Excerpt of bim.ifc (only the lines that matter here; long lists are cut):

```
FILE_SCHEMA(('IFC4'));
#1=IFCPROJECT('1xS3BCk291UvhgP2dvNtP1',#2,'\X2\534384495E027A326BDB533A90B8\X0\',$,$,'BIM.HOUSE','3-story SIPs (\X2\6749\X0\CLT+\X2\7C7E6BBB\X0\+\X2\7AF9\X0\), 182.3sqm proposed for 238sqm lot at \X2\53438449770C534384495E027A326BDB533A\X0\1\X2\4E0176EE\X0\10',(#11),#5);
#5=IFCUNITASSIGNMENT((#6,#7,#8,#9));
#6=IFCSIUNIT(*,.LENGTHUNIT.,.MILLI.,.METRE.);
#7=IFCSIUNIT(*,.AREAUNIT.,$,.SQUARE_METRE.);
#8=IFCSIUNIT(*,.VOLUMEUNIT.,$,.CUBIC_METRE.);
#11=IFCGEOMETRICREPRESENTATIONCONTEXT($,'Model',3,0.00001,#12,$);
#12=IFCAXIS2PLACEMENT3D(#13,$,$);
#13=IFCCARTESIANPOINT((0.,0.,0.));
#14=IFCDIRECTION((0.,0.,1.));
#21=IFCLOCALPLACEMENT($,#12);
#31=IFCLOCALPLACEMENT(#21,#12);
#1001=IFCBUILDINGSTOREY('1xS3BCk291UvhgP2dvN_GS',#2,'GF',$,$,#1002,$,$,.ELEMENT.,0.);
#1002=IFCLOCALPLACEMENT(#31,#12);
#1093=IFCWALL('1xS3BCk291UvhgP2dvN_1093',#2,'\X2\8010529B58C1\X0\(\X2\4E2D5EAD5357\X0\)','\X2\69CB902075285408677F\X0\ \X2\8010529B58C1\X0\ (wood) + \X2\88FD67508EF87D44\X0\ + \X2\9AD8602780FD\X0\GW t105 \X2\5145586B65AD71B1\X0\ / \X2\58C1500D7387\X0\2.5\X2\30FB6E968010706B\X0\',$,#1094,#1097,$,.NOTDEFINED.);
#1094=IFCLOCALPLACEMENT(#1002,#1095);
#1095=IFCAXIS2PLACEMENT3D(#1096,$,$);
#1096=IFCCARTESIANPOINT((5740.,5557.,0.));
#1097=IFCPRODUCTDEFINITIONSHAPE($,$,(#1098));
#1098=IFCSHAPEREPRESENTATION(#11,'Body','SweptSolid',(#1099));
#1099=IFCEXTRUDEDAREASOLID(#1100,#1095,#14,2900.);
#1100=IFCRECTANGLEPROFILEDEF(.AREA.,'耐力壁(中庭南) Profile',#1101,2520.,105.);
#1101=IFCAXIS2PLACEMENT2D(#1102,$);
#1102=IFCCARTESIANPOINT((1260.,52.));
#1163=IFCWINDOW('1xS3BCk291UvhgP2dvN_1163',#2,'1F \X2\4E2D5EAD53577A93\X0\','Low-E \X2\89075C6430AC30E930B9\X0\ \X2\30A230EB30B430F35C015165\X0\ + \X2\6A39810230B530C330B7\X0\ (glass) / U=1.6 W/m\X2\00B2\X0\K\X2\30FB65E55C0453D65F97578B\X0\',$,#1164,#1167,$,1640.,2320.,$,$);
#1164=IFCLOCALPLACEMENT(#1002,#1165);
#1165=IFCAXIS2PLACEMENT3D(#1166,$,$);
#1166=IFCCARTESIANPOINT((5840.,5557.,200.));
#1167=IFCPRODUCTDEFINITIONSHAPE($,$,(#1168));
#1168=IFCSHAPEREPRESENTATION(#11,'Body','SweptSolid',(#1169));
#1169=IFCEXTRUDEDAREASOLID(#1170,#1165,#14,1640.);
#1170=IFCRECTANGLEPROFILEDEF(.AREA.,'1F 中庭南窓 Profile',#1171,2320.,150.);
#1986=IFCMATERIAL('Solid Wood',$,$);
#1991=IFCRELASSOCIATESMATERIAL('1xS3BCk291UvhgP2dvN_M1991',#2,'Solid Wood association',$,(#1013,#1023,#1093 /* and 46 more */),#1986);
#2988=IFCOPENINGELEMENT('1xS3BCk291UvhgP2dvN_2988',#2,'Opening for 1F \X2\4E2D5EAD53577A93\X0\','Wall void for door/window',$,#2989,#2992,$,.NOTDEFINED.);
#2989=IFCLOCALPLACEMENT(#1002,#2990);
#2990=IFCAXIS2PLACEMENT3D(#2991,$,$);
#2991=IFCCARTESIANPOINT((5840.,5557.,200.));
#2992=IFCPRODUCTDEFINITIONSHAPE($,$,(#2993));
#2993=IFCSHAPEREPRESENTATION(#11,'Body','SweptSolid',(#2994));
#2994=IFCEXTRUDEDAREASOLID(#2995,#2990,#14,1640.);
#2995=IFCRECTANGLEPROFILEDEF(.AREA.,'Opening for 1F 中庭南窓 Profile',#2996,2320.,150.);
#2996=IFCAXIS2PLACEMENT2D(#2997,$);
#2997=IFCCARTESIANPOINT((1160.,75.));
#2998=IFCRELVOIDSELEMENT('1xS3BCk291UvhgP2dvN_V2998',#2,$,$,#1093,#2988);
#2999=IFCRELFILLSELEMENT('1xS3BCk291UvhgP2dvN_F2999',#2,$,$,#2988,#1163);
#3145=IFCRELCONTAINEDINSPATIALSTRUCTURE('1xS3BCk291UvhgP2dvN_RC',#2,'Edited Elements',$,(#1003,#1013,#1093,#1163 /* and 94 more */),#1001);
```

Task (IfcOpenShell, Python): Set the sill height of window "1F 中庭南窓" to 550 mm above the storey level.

```python
import numpy as np
import ifcopenshell
import ifcopenshell.api.geometry
import ifcopenshell.geom
import ifcopenshell.util.element
import ifcopenshell.util.placement
import ifcopenshell.util.shape
import ifcopenshell.util.unit

model = ifcopenshell.open("bim.ifc")
unit_scale = ifcopenshell.util.unit.calculate_unit_scale(model)

window = model.by_guid("1xS3BCk291UvhgP2dvN_1163")
opening = window.FillsVoids[0].RelatingOpeningElement
storey = ifcopenshell.util.element.get_container(window, ifc_class="IfcBuildingStorey")
level = ifcopenshell.util.placement.get_local_placement(storey.ObjectPlacement)[2, 3]

# The opening's origin need not be at the sill, so measure its lowest point.
shape = ifcopenshell.geom.create_shape(ifcopenshell.geom.settings(), opening)
bottom = ifcopenshell.util.shape.get_shape_bottom_elevation(shape, shape.geometry) / unit_scale
dz = level + 550.0 - bottom

shift = np.array([0.0, 0.0, dz])
# The window is not placed relative to its opening, so move both.
for product in (opening, window):
    matrix = ifcopenshell.util.placement.get_local_placement(product.ObjectPlacement)
    matrix[:3, 3] += shift
    ifcopenshell.api.geometry.edit_object_placement(model, product=product, matrix=matrix, is_si=False)

print(f"moved by {dz * unit_scale:+.3f} m")

model.write("bim_rev.ifc")
```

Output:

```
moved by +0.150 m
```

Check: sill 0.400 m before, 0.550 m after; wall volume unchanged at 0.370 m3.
